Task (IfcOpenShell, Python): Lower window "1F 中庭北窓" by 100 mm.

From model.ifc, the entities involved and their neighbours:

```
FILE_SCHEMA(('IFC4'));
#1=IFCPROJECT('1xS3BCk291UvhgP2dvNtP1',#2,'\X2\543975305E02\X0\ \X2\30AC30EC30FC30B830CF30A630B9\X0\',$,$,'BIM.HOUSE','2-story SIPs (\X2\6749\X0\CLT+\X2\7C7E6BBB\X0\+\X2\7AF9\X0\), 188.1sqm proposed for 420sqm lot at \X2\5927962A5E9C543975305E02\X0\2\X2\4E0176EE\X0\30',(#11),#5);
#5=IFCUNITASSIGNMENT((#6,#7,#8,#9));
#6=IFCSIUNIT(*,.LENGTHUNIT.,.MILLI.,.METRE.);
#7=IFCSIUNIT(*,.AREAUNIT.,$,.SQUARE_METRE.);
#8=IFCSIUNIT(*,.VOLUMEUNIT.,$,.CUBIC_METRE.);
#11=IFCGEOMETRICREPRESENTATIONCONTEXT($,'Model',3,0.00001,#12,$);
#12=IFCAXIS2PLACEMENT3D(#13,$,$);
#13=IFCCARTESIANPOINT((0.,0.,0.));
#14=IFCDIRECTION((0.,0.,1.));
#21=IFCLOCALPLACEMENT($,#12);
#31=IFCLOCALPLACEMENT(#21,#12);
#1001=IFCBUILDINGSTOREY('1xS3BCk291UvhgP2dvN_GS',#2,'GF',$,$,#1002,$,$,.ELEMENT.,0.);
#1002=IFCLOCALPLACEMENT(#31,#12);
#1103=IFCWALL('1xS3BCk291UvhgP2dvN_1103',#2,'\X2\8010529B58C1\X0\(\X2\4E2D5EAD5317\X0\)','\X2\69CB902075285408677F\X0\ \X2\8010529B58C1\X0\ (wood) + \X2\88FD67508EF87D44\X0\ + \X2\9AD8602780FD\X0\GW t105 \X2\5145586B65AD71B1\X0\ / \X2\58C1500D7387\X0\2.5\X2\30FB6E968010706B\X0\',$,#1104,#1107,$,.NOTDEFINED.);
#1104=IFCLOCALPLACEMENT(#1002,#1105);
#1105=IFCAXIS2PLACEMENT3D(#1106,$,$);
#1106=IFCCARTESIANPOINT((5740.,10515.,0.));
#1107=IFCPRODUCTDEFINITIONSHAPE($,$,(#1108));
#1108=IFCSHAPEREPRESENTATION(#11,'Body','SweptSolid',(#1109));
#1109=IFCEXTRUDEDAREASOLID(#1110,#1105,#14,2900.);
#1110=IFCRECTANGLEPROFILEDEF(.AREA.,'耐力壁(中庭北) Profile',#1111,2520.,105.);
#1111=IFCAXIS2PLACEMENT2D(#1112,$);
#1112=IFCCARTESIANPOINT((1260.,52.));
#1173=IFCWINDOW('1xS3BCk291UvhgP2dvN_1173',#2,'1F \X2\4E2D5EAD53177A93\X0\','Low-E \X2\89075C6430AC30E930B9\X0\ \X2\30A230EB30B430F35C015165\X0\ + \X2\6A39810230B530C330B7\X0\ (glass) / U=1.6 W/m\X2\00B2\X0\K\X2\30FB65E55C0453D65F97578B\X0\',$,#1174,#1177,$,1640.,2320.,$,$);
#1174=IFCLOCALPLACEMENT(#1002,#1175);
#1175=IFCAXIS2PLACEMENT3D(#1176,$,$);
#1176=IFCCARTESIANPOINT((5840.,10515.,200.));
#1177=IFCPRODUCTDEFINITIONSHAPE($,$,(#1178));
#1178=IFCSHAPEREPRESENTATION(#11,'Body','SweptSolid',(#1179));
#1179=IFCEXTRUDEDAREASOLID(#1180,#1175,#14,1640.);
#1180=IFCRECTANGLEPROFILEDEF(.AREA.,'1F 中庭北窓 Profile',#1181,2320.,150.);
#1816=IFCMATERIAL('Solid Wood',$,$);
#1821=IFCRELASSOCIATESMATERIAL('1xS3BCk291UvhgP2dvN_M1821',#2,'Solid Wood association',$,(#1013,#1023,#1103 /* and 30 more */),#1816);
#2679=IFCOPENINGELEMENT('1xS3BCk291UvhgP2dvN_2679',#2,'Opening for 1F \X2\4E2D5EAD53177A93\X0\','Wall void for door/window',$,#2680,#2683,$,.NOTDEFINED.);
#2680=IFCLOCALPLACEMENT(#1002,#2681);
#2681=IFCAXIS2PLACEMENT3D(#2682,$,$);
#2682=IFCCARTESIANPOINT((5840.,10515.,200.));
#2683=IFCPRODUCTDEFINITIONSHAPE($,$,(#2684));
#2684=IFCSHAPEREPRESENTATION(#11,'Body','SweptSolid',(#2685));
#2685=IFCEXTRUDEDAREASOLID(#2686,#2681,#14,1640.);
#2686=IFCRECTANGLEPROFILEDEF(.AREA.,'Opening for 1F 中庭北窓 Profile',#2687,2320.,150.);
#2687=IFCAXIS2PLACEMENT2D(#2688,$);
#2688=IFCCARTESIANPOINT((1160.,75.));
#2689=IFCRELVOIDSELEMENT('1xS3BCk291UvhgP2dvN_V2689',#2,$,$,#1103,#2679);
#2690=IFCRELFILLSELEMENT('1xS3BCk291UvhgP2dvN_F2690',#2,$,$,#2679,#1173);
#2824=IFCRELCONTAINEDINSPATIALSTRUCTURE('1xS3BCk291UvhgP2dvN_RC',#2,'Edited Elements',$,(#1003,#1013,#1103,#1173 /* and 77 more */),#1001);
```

```python
import numpy as np
import ifcopenshell
import ifcopenshell.api.geometry
import ifcopenshell.util.placement
import ifcopenshell.util.unit

model = ifcopenshell.open("model.ifc")
unit_scale = ifcopenshell.util.unit.calculate_unit_scale(model)

window = model.by_guid("1xS3BCk291UvhgP2dvN_1173")
opening = window.FillsVoids[0].RelatingOpeningElement
dz = -100.0

shift = np.array([0.0, 0.0, dz])
# The window is not placed relative to its opening, so move both.
for product in (opening, window):
    matrix = ifcopenshell.util.placement.get_local_placement(product.ObjectPlacement)
    matrix[:3, 3] += shift
    ifcopenshell.api.geometry.edit_object_placement(model, product=product, matrix=matrix, is_si=False)

print(f"moved by {dz * unit_scale:+.3f} m")

model.write("model_updated.ifc")
```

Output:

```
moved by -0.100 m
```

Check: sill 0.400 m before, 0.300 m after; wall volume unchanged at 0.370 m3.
